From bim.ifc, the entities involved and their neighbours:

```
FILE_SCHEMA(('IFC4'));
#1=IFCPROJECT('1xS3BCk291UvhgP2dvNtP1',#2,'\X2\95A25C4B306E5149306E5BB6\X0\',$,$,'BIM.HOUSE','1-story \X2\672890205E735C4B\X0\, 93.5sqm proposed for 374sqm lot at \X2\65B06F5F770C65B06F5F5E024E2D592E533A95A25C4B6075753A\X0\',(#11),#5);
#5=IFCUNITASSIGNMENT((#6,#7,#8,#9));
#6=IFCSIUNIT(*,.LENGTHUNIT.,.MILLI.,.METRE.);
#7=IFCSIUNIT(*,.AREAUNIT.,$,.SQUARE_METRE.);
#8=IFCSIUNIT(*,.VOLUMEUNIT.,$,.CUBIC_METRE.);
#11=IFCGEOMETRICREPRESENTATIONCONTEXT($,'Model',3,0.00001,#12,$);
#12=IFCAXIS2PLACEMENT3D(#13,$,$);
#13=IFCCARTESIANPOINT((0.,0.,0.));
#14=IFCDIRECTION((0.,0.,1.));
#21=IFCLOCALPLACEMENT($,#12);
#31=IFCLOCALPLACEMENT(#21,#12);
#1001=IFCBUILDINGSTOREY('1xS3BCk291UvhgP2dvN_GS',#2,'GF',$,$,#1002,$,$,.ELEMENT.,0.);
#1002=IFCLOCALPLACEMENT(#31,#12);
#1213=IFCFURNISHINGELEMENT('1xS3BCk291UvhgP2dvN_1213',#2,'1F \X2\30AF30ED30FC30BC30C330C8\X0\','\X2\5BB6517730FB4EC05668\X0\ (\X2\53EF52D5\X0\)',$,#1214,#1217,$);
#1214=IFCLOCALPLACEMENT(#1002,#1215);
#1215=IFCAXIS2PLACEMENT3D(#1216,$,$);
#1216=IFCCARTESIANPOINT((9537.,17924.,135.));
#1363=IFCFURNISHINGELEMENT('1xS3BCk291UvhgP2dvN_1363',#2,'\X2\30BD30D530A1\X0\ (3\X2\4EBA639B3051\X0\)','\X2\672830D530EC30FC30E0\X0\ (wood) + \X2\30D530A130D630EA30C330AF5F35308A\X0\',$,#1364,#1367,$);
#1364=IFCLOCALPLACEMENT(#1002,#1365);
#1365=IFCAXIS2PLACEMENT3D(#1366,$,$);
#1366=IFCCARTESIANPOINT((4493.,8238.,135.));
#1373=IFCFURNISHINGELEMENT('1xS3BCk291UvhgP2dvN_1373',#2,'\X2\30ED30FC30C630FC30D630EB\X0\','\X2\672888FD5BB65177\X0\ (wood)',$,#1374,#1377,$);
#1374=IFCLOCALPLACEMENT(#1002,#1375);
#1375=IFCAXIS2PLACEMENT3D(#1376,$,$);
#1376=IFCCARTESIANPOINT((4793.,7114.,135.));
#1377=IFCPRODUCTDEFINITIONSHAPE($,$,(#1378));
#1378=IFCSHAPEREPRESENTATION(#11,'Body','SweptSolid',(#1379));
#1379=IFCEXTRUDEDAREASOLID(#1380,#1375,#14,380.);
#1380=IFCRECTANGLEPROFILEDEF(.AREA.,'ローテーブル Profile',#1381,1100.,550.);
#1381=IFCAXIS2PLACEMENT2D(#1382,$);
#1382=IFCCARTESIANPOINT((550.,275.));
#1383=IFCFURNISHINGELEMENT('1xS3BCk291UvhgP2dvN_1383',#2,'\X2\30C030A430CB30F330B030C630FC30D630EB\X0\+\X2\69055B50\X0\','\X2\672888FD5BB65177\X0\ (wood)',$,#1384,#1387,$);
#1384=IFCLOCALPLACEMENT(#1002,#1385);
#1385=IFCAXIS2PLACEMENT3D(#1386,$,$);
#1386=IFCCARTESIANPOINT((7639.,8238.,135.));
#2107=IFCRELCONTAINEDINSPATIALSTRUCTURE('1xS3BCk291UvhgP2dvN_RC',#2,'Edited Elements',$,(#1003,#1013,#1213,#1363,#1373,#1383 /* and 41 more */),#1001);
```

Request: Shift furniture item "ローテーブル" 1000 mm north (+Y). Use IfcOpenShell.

```python
import ifcopenshell
import ifcopenshell.api.geometry
import ifcopenshell.util.placement

model = ifcopenshell.open("bim.ifc")

item = model.by_guid("1xS3BCk291UvhgP2dvN_1373")
matrix = ifcopenshell.util.placement.get_local_placement(item.ObjectPlacement)
matrix[1, 3] += 1000.0
ifcopenshell.api.geometry.edit_object_placement(model, product=item, matrix=matrix, is_si=False)

print(ifcopenshell.util.placement.get_local_placement(item.ObjectPlacement).round(3) + 0.0)

model.write("bim_rev.ifc")
```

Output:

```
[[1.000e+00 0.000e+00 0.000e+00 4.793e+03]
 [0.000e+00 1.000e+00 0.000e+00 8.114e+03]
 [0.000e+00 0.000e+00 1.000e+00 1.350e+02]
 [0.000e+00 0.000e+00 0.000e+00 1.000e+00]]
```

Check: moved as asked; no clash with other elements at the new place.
